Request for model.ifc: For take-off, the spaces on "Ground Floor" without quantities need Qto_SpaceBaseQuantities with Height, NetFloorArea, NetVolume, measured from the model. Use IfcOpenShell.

First a look at what the model holds.

```python
import ifcopenshell
import ifcopenshell.util.element
import ifcopenshell.util.unit

model = ifcopenshell.open("model.ifc")
print(model.schema)
for unit_type in ("LENGTHUNIT", "AREAUNIT", "VOLUMEUNIT"):
    print(unit_type, ifcopenshell.util.unit.calculate_unit_scale(model, unit_type))
storey = next(s for s in model.by_type("IfcBuildingStorey") if s.Name == "Ground Floor")
spaces = [e for e in ifcopenshell.util.element.get_decomposition(storey) if e.is_a("IfcSpace")]
for e in sorted(spaces, key=lambda e: e.id()):
    print(e.id(), e.is_a(), e.Name, list(ifcopenshell.util.element.get_psets(e, qtos_only=True)), sep=" | ")
```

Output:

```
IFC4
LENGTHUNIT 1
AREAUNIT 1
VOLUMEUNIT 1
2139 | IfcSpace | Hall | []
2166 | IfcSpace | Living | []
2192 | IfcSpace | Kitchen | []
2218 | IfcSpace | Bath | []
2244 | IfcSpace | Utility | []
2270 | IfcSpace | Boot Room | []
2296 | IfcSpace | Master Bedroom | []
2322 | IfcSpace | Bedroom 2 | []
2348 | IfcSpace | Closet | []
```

```python
import ifcopenshell
import ifcopenshell.api.pset
import ifcopenshell.geom
import ifcopenshell.util.element
import ifcopenshell.util.shape
import ifcopenshell.util.unit

model = ifcopenshell.open("model.ifc")
unit_scale = ifcopenshell.util.unit.calculate_unit_scale(model)
area_scale = ifcopenshell.util.unit.calculate_unit_scale(model, "AREAUNIT")
volume_scale = ifcopenshell.util.unit.calculate_unit_scale(model, "VOLUMEUNIT")
settings = ifcopenshell.geom.settings()

storey = next(s for s in model.by_type("IfcBuildingStorey") if s.Name == "Ground Floor")
spaces = [e for e in ifcopenshell.util.element.get_decomposition(storey) if e.is_a("IfcSpace")]

for e in sorted(spaces, key=lambda e: e.id()):
    if ifcopenshell.util.element.get_psets(e, qtos_only=True, should_inherit=False):
        continue
    # Geometry comes back in metres, in the element's own axes.
    shape = ifcopenshell.geom.create_shape(settings, e)
    values = {
        "Height": ifcopenshell.util.shape.get_z(shape.geometry) / unit_scale,
        "NetFloorArea": ifcopenshell.util.shape.get_footprint_area(shape.geometry) / area_scale,
        "NetVolume": ifcopenshell.util.shape.get_volume(shape.geometry) / volume_scale,
    }
    qto = ifcopenshell.api.pset.add_qto(model, product=e, name="Qto_SpaceBaseQuantities")
    ifcopenshell.api.pset.edit_qto(model, qto=qto, properties=values)
    print(e.id(), {k: round(v, 3) for k, v in values.items()})

model.write("model_updated.ifc")
```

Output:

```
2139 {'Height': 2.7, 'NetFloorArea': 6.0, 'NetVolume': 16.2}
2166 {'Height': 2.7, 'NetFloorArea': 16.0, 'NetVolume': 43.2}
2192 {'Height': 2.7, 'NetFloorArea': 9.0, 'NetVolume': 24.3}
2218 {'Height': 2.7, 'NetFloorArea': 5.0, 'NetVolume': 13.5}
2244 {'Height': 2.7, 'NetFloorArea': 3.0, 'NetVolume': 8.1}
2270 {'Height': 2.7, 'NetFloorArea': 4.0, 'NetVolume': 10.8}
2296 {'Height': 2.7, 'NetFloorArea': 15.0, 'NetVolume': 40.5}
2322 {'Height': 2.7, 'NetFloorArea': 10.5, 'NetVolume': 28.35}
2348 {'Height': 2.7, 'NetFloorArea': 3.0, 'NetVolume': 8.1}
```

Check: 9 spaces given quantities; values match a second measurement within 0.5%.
